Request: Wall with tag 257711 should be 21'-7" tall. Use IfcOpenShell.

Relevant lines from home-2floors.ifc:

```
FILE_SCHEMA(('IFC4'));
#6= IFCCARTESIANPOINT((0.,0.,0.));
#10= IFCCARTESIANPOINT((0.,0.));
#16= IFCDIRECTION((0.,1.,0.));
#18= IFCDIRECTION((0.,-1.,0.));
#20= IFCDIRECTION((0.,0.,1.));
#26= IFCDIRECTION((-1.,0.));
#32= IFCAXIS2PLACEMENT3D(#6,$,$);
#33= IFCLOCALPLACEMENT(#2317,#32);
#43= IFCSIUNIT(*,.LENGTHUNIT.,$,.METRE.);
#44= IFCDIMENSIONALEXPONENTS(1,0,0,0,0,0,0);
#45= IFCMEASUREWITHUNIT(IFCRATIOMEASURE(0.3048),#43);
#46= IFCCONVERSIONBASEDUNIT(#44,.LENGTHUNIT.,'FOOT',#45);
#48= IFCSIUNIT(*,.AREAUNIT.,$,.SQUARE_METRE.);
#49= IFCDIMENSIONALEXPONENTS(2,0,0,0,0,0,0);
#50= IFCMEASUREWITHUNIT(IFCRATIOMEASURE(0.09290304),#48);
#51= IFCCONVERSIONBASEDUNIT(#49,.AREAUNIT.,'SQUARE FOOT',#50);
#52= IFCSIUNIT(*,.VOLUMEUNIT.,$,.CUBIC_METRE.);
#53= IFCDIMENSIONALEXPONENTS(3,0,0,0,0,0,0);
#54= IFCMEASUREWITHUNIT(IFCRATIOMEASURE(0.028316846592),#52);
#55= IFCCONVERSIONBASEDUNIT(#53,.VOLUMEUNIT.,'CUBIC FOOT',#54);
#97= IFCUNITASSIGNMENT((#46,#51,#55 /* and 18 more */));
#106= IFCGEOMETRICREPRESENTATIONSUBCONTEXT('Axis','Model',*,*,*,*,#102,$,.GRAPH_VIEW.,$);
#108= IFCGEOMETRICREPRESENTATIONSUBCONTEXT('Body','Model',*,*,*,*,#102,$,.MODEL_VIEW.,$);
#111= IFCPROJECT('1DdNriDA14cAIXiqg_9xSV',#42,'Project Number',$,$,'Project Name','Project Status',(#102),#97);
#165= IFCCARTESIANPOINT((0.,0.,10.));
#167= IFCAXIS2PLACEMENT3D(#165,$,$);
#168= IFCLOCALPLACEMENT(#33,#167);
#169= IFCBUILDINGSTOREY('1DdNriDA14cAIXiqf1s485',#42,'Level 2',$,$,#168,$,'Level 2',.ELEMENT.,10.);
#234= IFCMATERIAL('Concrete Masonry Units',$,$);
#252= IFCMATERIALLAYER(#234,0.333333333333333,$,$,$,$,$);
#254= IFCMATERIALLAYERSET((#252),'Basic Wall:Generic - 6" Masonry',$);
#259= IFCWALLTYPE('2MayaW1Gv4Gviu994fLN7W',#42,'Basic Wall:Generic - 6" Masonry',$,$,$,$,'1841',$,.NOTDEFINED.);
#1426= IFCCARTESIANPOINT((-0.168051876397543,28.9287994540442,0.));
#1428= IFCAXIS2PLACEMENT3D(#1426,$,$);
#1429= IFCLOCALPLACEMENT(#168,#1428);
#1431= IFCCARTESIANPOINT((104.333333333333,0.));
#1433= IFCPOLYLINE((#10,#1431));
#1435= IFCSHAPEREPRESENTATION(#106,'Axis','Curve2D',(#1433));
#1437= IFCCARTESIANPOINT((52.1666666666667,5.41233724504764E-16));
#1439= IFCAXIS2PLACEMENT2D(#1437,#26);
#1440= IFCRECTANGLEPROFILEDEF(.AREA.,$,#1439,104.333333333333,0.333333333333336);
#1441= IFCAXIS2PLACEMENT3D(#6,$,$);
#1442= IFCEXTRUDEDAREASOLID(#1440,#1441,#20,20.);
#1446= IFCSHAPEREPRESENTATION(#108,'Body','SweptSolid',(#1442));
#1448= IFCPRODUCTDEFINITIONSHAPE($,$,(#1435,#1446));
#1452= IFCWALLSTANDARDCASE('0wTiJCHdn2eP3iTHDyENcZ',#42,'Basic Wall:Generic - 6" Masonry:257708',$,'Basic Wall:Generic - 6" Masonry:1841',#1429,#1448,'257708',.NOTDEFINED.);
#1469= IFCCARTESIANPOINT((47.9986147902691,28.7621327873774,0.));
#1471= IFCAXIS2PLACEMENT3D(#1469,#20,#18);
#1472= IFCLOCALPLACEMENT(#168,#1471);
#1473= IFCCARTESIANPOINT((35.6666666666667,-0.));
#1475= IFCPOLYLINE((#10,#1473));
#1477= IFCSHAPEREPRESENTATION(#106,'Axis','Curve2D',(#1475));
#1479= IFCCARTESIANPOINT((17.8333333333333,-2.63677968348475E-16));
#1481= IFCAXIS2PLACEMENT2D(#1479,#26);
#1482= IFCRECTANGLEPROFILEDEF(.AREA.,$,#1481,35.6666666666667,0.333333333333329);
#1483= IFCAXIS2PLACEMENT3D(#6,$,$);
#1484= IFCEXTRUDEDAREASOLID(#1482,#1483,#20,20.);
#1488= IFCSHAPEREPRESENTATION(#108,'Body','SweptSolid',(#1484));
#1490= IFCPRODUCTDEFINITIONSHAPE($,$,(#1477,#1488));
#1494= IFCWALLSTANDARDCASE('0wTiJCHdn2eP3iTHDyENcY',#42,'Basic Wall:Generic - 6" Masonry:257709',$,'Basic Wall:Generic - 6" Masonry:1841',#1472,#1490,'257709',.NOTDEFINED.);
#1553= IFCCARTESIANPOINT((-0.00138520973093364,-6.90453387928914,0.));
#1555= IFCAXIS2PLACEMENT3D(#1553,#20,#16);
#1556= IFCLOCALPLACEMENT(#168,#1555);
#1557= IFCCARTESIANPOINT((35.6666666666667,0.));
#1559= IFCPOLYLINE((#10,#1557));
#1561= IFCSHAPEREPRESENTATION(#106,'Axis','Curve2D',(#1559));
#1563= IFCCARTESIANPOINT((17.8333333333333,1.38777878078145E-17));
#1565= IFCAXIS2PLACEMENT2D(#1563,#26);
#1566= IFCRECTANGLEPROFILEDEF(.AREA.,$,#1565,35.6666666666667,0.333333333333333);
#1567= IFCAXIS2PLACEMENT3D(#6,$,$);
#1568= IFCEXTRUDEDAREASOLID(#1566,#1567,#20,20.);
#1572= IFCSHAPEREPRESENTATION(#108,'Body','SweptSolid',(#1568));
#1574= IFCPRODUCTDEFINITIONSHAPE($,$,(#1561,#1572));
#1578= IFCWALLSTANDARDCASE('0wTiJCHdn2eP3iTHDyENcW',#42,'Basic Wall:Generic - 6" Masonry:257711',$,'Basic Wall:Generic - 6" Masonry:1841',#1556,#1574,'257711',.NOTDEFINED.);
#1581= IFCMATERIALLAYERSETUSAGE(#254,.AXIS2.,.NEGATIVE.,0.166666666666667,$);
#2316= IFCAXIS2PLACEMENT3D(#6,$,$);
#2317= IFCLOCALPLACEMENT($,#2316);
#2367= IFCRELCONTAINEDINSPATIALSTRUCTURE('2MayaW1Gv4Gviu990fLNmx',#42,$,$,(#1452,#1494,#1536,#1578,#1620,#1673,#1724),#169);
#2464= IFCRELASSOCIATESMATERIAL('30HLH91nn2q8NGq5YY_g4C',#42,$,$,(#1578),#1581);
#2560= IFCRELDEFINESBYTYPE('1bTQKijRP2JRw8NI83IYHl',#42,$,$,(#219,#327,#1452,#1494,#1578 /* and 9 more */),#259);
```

```python
import ifcopenshell
import ifcopenshell.geom
import ifcopenshell.util.representation
import ifcopenshell.util.shape
import ifcopenshell.util.unit

model = ifcopenshell.open("home-2floors.ifc")
unit_scale = ifcopenshell.util.unit.calculate_unit_scale(model)
settings = ifcopenshell.geom.settings()


def volume(element):
    """Net volume in cubic metres, openings subtracted."""
    shape = ifcopenshell.geom.create_shape(settings, element)
    return ifcopenshell.util.shape.get_volume(shape.geometry)


wall = model.by_id(1578)
before = volume(wall)

body = ifcopenshell.util.representation.get_representation(wall, "Model", "Body")
solid = body.Items[0]
old_height = solid.Depth
solid.Depth = 259 * 0.0254 / unit_scale
after = volume(wall)

print(f"height {old_height:g} -> {solid.Depth:g}, volume {before:.3f} -> {after:.3f} m3")

model.write("home-2floors_updated.ifc")
```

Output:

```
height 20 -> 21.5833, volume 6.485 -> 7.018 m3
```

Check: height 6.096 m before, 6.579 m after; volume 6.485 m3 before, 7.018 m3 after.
